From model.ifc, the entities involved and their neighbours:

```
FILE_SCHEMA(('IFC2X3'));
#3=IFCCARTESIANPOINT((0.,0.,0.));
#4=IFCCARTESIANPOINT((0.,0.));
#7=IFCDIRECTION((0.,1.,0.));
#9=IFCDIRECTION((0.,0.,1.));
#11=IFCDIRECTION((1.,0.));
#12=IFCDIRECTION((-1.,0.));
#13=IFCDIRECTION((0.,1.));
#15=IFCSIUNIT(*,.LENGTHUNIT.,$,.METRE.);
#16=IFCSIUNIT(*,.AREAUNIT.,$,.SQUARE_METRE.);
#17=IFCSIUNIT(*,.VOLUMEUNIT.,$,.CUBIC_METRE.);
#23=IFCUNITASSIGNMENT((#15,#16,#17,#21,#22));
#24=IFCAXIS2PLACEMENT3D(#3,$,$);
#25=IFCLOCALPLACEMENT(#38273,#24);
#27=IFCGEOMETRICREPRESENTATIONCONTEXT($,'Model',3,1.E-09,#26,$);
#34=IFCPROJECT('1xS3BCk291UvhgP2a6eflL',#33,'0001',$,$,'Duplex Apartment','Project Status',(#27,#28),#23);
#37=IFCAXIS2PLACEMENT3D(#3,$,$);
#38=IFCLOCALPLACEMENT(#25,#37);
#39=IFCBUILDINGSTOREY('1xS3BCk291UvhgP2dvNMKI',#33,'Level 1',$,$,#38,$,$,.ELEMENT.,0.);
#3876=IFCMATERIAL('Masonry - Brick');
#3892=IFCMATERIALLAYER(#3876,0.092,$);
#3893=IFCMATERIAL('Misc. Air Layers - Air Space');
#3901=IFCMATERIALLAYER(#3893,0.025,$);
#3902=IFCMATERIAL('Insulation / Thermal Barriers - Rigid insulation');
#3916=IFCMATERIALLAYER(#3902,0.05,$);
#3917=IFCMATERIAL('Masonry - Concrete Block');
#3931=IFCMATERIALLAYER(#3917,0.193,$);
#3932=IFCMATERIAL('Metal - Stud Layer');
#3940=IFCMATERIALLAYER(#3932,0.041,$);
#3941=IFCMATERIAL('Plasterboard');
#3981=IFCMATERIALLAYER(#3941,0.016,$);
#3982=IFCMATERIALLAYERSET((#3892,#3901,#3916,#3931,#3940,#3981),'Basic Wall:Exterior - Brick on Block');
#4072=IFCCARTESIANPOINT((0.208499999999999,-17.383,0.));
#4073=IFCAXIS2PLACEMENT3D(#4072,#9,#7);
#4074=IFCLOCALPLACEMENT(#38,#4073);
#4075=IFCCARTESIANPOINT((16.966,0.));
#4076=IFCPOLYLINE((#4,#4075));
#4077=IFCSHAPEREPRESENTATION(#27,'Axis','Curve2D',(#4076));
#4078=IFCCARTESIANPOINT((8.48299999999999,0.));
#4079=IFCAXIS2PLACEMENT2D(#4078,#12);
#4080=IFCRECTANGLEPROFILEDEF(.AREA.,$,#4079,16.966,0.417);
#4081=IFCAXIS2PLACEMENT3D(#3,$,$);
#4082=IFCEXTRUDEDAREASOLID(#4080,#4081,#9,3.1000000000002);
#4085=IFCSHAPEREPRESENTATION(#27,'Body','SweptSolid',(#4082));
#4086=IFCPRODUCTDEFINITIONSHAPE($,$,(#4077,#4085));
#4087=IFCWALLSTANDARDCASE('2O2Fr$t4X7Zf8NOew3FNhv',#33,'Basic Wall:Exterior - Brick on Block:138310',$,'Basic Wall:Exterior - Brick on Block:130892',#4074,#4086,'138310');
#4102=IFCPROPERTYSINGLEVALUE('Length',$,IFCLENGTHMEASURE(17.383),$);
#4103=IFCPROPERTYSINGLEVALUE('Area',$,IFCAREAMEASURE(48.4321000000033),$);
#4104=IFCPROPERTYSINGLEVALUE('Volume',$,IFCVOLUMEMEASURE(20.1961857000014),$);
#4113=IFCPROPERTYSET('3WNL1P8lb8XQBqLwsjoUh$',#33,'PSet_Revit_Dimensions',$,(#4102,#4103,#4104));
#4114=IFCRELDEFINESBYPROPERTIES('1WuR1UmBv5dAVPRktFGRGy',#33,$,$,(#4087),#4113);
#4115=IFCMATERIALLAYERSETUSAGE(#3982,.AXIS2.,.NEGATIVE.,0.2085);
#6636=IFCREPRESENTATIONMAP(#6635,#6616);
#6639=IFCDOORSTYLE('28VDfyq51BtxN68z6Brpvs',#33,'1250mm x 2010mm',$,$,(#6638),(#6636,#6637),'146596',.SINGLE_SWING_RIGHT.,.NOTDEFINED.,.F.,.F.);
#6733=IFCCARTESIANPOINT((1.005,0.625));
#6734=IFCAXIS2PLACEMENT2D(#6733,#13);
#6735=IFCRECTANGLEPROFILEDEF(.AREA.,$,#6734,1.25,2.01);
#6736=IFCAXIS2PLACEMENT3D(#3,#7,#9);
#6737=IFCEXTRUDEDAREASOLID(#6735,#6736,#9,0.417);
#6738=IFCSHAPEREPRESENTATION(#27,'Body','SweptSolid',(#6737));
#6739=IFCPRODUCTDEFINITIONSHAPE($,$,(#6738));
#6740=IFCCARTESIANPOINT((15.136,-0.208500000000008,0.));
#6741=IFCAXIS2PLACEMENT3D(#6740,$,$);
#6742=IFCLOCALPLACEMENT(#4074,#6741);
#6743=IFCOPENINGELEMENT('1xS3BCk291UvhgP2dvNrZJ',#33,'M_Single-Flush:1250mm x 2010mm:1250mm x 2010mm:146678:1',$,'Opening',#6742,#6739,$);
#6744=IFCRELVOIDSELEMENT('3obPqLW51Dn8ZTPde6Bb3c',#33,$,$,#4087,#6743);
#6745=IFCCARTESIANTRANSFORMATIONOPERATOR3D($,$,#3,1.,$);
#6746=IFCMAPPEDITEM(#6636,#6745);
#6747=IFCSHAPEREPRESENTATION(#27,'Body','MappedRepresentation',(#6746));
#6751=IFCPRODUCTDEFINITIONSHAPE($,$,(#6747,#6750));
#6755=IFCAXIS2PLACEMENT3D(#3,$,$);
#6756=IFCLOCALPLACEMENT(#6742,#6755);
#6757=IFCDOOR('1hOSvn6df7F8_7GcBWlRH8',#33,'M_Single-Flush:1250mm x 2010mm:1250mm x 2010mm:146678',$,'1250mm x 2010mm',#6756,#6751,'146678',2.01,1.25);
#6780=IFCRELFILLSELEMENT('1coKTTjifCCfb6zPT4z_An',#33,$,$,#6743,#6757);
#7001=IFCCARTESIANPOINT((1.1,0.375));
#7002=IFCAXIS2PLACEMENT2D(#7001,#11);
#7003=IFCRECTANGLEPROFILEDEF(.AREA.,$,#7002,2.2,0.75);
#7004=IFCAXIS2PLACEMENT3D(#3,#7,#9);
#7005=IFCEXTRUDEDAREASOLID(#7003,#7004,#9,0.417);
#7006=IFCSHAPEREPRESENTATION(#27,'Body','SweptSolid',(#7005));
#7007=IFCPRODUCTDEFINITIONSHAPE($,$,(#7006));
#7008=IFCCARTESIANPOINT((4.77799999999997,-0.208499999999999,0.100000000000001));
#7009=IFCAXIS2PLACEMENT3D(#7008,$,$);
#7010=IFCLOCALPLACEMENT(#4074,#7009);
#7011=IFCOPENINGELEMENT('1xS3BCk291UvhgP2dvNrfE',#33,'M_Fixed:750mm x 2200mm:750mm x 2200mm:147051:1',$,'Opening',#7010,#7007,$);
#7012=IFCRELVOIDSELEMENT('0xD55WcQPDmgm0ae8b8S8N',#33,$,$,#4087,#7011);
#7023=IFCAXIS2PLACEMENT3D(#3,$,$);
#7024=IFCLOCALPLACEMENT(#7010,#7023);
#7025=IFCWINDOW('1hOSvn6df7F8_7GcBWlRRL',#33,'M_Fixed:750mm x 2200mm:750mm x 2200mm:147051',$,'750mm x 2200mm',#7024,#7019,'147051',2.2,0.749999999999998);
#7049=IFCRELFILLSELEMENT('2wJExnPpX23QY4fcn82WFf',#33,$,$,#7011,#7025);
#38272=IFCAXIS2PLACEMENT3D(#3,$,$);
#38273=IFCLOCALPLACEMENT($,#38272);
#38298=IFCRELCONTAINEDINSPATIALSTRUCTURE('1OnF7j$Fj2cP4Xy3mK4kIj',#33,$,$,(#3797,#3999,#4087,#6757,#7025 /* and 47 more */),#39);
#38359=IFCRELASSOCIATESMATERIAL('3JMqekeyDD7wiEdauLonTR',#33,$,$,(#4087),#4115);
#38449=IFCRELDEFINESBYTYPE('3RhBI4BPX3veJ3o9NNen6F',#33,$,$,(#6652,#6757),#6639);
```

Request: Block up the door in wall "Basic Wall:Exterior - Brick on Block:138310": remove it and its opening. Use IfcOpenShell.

```python
import ifcopenshell
import ifcopenshell.api.feature
import ifcopenshell.api.pset
import ifcopenshell.api.root
import ifcopenshell.geom
import ifcopenshell.util.element
import ifcopenshell.util.shape
import ifcopenshell.util.unit

model = ifcopenshell.open("model.ifc")
area_scale = ifcopenshell.util.unit.calculate_unit_scale(model, "AREAUNIT")
volume_scale = ifcopenshell.util.unit.calculate_unit_scale(model, "VOLUMEUNIT")
settings = ifcopenshell.geom.settings()


def volume(element):
    """Net volume in cubic metres, openings subtracted."""
    shape = ifcopenshell.geom.create_shape(settings, element)
    return ifcopenshell.util.shape.get_volume(shape.geometry)


door = model.by_guid("1hOSvn6df7F8_7GcBWlRH8")
opening = door.FillsVoids[0].RelatingOpeningElement
wall = opening.VoidsElements[0].RelatingBuildingElement
before = volume(wall)

ifcopenshell.api.root.remove_product(model, product=door)
ifcopenshell.api.feature.remove_feature(model, feature=opening)

after = volume(wall)
thickness = 0.417  # wall thickness in metres

# Update the wall's stored quantities.
pset = model.by_id(ifcopenshell.util.element.get_pset(wall, "PSet_Revit_Dimensions", should_inherit=False)["id"])
ifcopenshell.api.pset.edit_pset(model, pset=pset, properties={
    "Area": model.create_entity("IfcAreaMeasure", after / thickness / area_scale),
    "Volume": model.create_entity("IfcVolumeMeasure", after / volume_scale),
})

print(f"wall volume {before:.3f} -> {after:.3f} m3")

model.write("model-out.ifc")
```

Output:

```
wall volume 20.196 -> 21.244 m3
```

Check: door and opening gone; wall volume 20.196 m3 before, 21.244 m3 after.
